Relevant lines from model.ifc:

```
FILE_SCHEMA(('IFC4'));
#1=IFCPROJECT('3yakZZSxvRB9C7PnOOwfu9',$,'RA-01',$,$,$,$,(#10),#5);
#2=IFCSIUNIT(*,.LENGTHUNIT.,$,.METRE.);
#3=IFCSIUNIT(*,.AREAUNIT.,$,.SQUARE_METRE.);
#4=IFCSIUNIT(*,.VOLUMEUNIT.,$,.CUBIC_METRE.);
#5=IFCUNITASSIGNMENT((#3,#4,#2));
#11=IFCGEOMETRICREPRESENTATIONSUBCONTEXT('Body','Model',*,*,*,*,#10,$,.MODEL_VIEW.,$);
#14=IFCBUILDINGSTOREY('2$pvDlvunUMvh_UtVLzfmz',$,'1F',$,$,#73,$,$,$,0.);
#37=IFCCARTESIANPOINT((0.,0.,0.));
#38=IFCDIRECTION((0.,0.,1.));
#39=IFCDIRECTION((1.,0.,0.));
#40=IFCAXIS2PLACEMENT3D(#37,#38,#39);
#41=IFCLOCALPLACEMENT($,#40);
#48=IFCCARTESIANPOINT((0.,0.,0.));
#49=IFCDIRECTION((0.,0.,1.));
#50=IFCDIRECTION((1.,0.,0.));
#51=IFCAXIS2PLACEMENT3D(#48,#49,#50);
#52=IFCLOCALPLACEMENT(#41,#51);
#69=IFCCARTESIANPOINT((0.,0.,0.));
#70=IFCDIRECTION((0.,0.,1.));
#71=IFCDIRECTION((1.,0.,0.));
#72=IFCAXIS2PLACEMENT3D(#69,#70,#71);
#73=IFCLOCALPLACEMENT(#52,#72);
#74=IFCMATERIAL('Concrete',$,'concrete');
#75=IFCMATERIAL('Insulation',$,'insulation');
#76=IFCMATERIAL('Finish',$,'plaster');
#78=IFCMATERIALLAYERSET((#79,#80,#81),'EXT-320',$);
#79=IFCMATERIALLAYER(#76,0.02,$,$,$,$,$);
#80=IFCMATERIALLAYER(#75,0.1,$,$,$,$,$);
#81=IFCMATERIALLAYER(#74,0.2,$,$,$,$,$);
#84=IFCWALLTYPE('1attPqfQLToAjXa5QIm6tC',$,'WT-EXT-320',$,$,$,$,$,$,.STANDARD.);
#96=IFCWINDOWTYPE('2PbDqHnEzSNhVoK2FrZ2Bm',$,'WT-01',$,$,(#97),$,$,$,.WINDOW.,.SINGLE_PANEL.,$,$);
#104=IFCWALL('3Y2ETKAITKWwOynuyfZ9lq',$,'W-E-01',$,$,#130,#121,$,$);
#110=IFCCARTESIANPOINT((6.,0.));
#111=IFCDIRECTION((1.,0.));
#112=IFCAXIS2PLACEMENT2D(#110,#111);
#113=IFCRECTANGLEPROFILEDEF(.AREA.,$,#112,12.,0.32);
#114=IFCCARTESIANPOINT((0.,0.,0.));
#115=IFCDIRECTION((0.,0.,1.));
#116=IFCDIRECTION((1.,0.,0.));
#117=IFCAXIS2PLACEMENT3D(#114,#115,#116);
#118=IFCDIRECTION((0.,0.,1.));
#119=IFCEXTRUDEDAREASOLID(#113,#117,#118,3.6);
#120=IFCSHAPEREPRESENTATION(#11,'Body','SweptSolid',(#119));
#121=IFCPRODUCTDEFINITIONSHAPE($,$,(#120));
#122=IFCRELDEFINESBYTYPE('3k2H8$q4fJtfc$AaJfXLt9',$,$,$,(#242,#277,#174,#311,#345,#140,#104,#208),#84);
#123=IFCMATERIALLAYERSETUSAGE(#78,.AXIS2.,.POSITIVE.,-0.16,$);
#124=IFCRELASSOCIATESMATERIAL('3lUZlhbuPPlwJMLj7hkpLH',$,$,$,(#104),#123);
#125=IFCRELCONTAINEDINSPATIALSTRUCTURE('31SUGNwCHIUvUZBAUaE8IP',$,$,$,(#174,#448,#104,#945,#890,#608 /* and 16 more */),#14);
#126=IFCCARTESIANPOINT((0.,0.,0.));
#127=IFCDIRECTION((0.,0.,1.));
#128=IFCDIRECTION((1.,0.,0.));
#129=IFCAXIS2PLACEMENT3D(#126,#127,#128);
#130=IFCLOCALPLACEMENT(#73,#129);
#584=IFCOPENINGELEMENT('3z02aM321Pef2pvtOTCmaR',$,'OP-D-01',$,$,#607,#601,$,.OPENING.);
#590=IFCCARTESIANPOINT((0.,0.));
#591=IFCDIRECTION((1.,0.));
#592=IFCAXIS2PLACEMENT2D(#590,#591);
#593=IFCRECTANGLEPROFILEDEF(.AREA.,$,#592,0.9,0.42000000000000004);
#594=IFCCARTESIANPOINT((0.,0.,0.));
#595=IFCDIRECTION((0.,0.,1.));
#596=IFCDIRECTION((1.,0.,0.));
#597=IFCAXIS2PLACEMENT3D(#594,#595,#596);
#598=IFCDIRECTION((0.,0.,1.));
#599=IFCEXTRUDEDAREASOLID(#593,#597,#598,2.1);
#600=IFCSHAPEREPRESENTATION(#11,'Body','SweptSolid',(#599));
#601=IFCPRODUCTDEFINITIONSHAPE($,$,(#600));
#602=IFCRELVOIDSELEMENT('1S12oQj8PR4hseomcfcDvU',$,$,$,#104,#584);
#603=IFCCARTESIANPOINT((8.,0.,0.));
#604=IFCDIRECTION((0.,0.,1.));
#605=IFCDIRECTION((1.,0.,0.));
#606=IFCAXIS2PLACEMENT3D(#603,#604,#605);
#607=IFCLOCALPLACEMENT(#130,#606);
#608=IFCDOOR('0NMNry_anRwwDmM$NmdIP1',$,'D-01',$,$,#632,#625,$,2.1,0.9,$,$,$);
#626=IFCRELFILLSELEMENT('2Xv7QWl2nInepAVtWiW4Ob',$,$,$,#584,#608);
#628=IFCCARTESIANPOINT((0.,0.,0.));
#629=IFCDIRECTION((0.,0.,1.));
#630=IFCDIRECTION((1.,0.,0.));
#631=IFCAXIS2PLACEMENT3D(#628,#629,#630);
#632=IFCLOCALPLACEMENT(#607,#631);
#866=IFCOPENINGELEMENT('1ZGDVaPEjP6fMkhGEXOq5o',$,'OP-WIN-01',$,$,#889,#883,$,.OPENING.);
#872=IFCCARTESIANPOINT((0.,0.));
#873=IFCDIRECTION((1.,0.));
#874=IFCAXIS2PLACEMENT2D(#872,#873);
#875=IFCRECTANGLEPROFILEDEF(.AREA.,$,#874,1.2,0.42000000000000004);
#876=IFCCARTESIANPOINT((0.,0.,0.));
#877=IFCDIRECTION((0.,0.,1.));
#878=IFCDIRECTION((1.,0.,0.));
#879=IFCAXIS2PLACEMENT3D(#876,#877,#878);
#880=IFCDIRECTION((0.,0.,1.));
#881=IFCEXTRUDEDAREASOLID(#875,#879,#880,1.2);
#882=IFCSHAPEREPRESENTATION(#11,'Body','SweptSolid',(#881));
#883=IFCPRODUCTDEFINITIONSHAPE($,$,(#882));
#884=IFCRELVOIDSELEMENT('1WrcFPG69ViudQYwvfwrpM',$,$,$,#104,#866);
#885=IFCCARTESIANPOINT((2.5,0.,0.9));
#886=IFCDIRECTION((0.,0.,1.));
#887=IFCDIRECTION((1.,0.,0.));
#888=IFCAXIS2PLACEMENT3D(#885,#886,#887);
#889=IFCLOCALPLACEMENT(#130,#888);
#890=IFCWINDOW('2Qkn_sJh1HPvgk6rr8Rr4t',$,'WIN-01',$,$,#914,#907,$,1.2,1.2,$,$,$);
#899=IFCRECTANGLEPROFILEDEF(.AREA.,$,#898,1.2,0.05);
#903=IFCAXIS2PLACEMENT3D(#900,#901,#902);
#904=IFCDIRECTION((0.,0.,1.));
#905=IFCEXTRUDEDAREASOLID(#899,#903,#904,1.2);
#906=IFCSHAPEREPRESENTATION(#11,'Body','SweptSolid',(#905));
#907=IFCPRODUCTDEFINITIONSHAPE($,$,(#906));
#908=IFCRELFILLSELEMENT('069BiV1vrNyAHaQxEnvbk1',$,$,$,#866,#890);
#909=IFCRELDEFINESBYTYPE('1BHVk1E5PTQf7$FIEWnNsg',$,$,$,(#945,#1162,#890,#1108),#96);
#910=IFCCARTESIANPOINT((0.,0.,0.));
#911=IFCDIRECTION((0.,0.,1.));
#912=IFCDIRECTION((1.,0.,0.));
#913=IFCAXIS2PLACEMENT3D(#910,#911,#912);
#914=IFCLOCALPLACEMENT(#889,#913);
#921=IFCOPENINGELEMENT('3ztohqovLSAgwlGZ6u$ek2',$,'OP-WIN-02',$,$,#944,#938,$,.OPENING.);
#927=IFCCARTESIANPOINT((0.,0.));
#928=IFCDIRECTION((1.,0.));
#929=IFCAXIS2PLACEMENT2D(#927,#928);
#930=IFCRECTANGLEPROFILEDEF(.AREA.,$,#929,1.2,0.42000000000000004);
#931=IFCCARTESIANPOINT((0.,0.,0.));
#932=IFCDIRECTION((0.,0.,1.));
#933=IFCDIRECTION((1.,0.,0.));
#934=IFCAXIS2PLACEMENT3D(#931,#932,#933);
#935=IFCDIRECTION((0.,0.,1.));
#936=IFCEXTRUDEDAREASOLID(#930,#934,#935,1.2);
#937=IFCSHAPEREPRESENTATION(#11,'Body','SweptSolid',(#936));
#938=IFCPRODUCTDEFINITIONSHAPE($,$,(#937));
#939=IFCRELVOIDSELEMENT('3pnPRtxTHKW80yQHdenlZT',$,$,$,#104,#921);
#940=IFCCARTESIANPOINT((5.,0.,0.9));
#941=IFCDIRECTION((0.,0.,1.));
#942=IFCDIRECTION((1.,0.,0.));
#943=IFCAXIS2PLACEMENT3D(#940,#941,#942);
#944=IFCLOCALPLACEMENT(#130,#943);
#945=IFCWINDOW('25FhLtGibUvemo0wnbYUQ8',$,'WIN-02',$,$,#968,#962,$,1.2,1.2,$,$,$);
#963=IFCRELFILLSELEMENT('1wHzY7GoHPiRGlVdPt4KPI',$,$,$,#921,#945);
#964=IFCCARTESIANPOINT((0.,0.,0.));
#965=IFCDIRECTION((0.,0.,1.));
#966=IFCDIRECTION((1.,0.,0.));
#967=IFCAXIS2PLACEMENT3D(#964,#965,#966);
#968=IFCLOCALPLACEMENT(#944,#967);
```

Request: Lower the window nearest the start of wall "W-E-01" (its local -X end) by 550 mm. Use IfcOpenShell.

```python
import numpy as np
import ifcopenshell
import ifcopenshell.api.geometry
import ifcopenshell.util.placement
import ifcopenshell.util.unit

model = ifcopenshell.open("model.ifc")
unit_scale = ifcopenshell.util.unit.calculate_unit_scale(model)

window = model.by_guid("2Qkn_sJh1HPvgk6rr8Rr4t")
opening = window.FillsVoids[0].RelatingOpeningElement
dz = -0.55 / unit_scale

shift = np.array([0.0, 0.0, dz])
# The window is placed relative to its opening, so it follows when the opening moves.
matrix = ifcopenshell.util.placement.get_local_placement(opening.ObjectPlacement)
matrix[:3, 3] += shift
ifcopenshell.api.geometry.edit_object_placement(
    model, product=opening, matrix=matrix, is_si=False, should_transform_children=True
)

print(f"moved by {dz * unit_scale:+.3f} m")

model.write("model_rev.ifc")
```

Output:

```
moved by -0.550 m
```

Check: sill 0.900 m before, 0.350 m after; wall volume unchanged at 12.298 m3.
